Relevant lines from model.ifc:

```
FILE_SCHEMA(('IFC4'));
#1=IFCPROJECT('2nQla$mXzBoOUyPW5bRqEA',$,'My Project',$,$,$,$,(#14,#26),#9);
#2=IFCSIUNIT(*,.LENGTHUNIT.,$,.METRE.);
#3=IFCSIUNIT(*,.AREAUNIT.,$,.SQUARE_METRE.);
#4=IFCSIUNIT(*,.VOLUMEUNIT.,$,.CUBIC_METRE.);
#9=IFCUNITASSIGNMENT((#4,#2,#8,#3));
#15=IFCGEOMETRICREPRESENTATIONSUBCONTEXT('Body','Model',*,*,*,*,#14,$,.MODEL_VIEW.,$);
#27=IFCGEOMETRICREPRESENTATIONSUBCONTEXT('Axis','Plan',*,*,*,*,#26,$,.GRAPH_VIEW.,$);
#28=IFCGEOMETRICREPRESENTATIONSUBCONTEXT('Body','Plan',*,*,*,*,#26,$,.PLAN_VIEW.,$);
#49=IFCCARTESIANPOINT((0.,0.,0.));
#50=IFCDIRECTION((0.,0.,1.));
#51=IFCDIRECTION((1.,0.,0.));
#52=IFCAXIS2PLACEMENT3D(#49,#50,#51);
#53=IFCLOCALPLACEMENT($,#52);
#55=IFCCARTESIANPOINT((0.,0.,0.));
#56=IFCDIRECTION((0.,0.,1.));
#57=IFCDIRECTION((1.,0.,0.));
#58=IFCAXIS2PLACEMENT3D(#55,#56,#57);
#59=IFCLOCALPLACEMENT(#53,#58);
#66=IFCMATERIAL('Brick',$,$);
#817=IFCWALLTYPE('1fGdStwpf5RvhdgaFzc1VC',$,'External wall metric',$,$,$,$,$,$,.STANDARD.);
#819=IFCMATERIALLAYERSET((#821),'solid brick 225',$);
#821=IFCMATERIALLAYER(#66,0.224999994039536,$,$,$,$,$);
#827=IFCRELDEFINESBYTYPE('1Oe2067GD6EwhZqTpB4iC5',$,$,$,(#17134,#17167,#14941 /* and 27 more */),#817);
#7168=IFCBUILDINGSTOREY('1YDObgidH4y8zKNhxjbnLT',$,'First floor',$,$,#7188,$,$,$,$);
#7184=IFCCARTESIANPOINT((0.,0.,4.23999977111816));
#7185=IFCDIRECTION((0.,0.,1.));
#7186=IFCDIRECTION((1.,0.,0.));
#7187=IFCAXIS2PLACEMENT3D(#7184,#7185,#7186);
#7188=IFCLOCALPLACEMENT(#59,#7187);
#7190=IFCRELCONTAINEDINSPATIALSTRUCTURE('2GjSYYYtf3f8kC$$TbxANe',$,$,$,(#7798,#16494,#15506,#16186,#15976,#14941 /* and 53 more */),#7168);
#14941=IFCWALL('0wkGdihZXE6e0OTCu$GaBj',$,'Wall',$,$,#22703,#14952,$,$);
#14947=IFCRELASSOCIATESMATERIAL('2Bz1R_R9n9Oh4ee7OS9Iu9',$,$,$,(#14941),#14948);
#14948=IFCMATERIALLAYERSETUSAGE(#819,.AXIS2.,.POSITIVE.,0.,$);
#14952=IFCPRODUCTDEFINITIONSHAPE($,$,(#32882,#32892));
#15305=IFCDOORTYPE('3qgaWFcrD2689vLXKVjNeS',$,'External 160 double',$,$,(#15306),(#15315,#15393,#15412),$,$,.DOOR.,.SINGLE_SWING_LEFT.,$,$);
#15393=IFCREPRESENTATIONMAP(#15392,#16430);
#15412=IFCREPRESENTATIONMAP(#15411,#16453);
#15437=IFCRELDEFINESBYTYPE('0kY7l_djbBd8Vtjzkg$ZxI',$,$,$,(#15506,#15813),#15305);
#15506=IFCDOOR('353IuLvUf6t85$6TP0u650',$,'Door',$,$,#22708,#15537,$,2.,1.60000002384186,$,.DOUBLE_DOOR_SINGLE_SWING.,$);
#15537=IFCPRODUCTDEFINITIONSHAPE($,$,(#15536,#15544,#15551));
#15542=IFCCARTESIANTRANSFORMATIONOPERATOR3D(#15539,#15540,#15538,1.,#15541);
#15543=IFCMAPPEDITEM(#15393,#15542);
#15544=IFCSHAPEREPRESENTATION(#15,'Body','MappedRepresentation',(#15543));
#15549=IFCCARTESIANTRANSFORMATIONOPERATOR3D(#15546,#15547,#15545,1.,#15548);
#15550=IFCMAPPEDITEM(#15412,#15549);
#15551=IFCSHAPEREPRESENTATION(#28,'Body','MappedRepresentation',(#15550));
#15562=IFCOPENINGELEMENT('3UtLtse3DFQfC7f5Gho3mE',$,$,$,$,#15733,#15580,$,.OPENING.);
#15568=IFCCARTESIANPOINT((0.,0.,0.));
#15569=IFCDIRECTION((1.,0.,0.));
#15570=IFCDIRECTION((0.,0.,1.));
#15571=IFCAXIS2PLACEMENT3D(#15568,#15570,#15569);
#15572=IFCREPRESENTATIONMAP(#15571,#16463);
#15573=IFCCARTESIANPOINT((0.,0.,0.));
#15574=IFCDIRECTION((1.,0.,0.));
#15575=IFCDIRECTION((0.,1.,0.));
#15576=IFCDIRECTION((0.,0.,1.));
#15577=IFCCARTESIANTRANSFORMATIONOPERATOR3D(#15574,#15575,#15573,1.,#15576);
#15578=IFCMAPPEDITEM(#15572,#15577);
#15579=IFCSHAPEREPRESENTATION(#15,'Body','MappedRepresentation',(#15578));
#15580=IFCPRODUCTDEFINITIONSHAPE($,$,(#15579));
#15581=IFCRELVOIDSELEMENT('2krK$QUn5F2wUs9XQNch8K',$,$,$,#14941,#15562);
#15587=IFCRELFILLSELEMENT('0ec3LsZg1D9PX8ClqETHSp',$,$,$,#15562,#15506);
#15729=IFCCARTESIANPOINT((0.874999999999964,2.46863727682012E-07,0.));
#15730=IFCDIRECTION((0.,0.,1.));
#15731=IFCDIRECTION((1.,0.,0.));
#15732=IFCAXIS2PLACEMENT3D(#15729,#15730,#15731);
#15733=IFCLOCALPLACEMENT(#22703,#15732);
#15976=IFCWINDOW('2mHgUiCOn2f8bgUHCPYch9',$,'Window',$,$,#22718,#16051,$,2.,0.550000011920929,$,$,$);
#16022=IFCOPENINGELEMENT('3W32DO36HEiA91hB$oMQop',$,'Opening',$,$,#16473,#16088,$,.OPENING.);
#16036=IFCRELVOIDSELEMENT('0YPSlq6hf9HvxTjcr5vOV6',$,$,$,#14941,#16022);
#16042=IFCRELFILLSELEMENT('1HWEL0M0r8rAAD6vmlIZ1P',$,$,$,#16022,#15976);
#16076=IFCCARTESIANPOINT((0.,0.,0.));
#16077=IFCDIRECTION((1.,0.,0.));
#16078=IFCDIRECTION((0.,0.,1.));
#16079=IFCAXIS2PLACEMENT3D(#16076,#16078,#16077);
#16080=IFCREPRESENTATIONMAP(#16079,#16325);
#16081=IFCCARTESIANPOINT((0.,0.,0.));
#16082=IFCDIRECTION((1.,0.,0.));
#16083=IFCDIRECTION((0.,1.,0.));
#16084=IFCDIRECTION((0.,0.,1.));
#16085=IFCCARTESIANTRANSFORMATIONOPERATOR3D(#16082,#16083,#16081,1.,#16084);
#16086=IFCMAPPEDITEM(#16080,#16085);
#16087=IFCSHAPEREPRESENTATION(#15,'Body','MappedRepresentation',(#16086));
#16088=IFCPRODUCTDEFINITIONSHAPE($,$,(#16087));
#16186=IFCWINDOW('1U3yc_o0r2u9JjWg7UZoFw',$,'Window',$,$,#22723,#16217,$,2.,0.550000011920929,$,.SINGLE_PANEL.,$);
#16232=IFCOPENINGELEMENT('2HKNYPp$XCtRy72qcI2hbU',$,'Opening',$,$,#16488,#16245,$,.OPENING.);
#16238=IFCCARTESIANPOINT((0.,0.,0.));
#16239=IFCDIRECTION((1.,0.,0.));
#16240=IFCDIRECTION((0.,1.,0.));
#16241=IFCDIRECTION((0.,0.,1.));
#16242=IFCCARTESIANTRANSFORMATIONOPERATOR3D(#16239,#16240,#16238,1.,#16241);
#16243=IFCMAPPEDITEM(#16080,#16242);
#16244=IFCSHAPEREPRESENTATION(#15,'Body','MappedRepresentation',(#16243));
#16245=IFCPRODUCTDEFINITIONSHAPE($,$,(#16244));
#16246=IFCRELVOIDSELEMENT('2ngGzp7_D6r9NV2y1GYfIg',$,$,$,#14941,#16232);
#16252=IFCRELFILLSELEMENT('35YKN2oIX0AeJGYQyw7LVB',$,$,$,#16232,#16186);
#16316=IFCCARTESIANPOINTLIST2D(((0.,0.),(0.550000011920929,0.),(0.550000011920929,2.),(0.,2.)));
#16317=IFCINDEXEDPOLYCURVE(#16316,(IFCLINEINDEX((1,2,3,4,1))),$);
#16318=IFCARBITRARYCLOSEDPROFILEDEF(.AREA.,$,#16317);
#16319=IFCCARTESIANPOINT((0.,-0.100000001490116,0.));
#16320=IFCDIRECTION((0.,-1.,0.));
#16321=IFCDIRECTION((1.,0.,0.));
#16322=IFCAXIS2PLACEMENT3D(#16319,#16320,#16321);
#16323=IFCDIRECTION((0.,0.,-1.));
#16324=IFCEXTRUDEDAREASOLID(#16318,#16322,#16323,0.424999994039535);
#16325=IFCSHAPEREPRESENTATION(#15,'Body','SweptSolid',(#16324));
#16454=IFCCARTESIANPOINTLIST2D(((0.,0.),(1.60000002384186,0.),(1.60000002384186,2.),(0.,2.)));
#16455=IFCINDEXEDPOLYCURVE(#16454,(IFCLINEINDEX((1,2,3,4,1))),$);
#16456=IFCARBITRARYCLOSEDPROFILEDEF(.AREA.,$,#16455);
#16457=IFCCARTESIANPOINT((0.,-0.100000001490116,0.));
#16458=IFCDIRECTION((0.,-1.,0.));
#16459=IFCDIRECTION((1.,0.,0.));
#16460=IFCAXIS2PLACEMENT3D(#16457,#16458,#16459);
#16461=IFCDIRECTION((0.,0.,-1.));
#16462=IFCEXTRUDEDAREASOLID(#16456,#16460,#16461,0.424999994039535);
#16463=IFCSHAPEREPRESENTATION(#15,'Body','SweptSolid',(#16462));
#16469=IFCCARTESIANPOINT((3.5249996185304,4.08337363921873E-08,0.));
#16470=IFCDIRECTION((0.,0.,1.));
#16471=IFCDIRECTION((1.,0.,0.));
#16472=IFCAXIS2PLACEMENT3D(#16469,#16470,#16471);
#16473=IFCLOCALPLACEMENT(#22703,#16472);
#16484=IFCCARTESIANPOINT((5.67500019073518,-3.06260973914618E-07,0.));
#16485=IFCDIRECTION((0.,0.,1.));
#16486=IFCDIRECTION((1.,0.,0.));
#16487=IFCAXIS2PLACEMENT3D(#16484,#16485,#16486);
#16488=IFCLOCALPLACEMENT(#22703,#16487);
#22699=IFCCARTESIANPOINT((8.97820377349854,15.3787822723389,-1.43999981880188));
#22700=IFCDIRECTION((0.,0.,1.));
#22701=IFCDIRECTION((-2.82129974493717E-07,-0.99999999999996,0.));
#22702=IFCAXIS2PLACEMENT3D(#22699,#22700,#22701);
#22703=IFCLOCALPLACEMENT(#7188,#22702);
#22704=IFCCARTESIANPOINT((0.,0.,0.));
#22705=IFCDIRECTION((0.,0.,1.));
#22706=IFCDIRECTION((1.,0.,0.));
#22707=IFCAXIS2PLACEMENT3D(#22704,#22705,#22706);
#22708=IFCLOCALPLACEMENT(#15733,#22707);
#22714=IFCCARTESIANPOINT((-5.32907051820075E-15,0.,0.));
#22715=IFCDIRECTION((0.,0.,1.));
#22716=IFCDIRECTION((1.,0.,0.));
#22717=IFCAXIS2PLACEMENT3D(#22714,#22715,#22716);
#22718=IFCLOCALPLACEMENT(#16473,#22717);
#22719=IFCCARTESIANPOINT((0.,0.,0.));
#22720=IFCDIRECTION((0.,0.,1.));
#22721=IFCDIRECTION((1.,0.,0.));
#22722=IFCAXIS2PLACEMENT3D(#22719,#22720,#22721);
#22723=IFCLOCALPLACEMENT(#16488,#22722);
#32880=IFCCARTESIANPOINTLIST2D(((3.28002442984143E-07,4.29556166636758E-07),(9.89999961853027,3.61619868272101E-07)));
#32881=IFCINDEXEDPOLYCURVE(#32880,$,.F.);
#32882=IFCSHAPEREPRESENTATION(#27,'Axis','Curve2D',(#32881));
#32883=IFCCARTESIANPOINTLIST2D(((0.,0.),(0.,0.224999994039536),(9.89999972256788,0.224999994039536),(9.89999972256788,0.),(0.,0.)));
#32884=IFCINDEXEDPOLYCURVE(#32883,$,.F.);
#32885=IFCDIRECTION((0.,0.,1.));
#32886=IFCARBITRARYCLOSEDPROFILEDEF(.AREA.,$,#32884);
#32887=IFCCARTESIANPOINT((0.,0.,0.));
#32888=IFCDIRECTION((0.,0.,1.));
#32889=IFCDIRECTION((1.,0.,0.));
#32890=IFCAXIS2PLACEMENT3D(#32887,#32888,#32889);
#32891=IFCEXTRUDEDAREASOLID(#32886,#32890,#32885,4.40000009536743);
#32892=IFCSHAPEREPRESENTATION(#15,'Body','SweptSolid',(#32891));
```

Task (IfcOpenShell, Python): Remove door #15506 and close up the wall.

```python
import ifcopenshell
import ifcopenshell.api.feature
import ifcopenshell.api.root
import ifcopenshell.geom
import ifcopenshell.util.shape

model = ifcopenshell.open("model.ifc")
settings = ifcopenshell.geom.settings()


def volume(element):
    """Net volume in cubic metres, openings subtracted."""
    shape = ifcopenshell.geom.create_shape(settings, element)
    return ifcopenshell.util.shape.get_volume(shape.geometry)


door = model.by_guid("353IuLvUf6t85$6TP0u650")
opening = door.FillsVoids[0].RelatingOpeningElement
wall = opening.VoidsElements[0].RelatingBuildingElement
before = volume(wall)

ifcopenshell.api.root.remove_product(model, product=door)
ifcopenshell.api.feature.remove_feature(model, feature=opening)

after = volume(wall)

print(f"wall volume {before:.3f} -> {after:.3f} m3")

model.write("model_v2.ifc")
```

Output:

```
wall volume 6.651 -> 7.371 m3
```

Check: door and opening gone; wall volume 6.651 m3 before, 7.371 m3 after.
